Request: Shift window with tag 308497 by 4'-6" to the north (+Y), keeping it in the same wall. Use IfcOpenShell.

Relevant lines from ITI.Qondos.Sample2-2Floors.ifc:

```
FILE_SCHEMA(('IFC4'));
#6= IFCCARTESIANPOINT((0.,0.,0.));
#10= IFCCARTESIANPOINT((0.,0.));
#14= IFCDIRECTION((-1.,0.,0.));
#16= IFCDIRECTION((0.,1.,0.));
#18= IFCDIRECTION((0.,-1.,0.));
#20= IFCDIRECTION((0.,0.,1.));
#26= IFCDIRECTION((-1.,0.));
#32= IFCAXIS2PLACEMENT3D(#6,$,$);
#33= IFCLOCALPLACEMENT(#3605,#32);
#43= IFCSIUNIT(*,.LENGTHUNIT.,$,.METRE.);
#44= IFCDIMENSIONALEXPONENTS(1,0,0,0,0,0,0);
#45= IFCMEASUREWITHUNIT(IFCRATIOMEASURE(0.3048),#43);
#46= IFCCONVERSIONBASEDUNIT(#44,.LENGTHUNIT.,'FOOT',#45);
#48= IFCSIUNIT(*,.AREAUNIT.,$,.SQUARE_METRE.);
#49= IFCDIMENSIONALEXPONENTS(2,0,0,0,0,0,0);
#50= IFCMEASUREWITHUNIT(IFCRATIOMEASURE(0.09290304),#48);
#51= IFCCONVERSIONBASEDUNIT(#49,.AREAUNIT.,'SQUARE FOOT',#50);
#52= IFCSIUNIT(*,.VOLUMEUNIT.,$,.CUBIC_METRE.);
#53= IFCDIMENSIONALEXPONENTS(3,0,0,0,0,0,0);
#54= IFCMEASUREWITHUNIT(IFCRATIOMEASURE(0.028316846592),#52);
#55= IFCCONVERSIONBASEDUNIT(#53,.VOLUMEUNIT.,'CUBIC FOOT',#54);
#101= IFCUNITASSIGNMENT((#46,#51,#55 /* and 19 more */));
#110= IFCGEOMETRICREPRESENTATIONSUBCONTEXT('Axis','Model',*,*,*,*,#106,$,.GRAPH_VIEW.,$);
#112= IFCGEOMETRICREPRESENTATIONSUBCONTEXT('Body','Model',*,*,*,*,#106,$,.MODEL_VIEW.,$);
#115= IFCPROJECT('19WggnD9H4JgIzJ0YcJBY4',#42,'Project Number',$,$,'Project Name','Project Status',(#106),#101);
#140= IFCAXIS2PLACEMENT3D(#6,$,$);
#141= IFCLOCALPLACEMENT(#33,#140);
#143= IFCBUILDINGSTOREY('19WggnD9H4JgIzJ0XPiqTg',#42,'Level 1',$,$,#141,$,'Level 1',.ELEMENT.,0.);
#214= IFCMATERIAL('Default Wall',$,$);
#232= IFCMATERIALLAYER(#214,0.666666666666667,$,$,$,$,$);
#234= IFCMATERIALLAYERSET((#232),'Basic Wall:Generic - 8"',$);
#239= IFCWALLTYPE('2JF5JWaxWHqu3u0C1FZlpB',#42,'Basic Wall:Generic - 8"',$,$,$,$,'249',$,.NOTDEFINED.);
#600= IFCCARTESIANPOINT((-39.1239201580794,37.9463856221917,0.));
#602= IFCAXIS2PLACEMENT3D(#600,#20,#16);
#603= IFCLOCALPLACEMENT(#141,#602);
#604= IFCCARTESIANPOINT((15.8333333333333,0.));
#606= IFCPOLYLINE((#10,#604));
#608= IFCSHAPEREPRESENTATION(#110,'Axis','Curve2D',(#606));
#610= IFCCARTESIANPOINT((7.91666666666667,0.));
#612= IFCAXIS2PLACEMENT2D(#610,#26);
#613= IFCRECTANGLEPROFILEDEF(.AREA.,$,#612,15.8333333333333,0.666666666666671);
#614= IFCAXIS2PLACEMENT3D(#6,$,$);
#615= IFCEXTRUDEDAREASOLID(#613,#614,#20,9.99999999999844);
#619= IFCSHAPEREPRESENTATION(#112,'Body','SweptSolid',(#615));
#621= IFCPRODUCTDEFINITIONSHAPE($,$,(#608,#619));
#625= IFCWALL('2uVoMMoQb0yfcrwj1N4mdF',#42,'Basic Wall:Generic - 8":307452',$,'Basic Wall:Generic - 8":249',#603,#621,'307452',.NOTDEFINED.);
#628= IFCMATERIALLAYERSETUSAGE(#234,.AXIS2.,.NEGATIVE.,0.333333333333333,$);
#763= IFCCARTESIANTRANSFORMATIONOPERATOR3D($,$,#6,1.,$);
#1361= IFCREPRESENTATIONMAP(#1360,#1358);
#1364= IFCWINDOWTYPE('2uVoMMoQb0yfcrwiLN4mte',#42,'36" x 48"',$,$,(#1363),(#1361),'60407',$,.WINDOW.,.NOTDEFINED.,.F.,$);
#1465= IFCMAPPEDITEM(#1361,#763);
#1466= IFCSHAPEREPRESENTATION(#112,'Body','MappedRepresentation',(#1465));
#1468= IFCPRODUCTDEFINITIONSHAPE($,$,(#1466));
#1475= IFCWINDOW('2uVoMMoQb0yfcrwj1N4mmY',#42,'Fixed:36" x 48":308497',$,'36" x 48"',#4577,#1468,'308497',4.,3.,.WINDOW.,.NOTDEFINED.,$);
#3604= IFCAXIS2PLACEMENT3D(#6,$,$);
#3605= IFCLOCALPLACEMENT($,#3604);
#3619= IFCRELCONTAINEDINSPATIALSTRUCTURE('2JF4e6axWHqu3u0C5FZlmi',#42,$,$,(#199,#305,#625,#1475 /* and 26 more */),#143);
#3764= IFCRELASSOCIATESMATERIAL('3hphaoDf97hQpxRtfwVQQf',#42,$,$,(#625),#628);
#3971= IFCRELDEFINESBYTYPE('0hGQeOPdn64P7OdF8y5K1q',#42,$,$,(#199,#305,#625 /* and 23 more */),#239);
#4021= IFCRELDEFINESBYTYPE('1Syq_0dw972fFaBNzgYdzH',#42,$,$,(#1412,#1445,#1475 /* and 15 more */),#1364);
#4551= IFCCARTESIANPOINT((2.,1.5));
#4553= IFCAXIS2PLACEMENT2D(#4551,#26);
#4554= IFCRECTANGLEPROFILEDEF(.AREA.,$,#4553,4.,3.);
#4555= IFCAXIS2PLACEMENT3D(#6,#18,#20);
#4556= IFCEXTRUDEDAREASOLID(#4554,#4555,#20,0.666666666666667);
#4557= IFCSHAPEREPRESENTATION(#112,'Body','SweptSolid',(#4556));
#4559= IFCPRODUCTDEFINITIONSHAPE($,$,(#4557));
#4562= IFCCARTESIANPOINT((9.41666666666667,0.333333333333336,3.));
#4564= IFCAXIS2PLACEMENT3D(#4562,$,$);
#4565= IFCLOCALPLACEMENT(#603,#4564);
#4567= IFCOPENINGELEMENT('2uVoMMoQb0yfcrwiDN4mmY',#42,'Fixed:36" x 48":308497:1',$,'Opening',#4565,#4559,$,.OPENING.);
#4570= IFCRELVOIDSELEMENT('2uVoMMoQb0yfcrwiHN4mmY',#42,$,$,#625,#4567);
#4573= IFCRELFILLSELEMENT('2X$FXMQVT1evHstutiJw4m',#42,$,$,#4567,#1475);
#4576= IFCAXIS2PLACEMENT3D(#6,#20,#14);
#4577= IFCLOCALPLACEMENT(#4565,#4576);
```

```python
import ifcopenshell
import ifcopenshell.api.geometry
import ifcopenshell.util.placement
import ifcopenshell.util.unit

model = ifcopenshell.open("ITI.Qondos.Sample2-2Floors.ifc")
unit_scale = ifcopenshell.util.unit.calculate_unit_scale(model)

window = model.by_id(1475)
opening = window.FillsVoids[0].RelatingOpeningElement
wall = opening.VoidsElements[0].RelatingBuildingElement

wall_matrix = ifcopenshell.util.placement.get_local_placement(wall.ObjectPlacement)
shift = wall_matrix[:3, 0] * 54 * 0.0254 / unit_scale
before = ifcopenshell.util.placement.get_local_placement(window.ObjectPlacement)[:3, 3].copy()

# The window is placed relative to its opening, so it follows when the opening moves.
matrix = ifcopenshell.util.placement.get_local_placement(opening.ObjectPlacement)
matrix[:3, 3] += shift
ifcopenshell.api.geometry.edit_object_placement(
    model, product=opening, matrix=matrix, is_si=False, should_transform_children=True
)

after = ifcopenshell.util.placement.get_local_placement(window.ObjectPlacement)[:3, 3]
print("window moved by", (after - before).round(3) + 0.0)

model.write("ITI.Qondos.Sample2-2Floors_v2.ifc")
```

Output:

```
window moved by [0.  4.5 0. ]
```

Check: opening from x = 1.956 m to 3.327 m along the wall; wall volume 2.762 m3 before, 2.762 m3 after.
